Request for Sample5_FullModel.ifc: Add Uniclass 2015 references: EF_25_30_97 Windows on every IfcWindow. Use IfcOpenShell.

First a look at what the model holds.

```python
import ifcopenshell

model = ifcopenshell.open("Sample5_FullModel.ifc")
print(model.schema)
print("classifications:", [c.Name for c in model.by_type("IfcClassification")])
for ifc_class in ("IfcDoor", "IfcRoof", "IfcStair", "IfcWall", "IfcWindow"):
    print(ifc_class, len(model.by_type(ifc_class)))
```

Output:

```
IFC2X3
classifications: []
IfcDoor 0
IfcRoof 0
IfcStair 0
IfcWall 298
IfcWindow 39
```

```python
import ifcopenshell
import ifcopenshell.api.classification

model = ifcopenshell.open("Sample5_FullModel.ifc")

# IFC2X3 requires Source and Edition and has no link from the project to the system.
system = model.create_entity("IfcClassification", Source="NBS", Edition="2015", Name="Uniclass 2015")

codes = {
    "IfcWindow": ("EF_25_30_97", "Windows"),
}
for ifc_class, (code, name) in codes.items():
    products = model.by_type(ifc_class)
    ifcopenshell.api.classification.add_reference(
        model, products=products, classification=system, identification=code, name=name
    )
    print(code, len(products))

model.write("Sample5_FullModel_rev.ifc")
```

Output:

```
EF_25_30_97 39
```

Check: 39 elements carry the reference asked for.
